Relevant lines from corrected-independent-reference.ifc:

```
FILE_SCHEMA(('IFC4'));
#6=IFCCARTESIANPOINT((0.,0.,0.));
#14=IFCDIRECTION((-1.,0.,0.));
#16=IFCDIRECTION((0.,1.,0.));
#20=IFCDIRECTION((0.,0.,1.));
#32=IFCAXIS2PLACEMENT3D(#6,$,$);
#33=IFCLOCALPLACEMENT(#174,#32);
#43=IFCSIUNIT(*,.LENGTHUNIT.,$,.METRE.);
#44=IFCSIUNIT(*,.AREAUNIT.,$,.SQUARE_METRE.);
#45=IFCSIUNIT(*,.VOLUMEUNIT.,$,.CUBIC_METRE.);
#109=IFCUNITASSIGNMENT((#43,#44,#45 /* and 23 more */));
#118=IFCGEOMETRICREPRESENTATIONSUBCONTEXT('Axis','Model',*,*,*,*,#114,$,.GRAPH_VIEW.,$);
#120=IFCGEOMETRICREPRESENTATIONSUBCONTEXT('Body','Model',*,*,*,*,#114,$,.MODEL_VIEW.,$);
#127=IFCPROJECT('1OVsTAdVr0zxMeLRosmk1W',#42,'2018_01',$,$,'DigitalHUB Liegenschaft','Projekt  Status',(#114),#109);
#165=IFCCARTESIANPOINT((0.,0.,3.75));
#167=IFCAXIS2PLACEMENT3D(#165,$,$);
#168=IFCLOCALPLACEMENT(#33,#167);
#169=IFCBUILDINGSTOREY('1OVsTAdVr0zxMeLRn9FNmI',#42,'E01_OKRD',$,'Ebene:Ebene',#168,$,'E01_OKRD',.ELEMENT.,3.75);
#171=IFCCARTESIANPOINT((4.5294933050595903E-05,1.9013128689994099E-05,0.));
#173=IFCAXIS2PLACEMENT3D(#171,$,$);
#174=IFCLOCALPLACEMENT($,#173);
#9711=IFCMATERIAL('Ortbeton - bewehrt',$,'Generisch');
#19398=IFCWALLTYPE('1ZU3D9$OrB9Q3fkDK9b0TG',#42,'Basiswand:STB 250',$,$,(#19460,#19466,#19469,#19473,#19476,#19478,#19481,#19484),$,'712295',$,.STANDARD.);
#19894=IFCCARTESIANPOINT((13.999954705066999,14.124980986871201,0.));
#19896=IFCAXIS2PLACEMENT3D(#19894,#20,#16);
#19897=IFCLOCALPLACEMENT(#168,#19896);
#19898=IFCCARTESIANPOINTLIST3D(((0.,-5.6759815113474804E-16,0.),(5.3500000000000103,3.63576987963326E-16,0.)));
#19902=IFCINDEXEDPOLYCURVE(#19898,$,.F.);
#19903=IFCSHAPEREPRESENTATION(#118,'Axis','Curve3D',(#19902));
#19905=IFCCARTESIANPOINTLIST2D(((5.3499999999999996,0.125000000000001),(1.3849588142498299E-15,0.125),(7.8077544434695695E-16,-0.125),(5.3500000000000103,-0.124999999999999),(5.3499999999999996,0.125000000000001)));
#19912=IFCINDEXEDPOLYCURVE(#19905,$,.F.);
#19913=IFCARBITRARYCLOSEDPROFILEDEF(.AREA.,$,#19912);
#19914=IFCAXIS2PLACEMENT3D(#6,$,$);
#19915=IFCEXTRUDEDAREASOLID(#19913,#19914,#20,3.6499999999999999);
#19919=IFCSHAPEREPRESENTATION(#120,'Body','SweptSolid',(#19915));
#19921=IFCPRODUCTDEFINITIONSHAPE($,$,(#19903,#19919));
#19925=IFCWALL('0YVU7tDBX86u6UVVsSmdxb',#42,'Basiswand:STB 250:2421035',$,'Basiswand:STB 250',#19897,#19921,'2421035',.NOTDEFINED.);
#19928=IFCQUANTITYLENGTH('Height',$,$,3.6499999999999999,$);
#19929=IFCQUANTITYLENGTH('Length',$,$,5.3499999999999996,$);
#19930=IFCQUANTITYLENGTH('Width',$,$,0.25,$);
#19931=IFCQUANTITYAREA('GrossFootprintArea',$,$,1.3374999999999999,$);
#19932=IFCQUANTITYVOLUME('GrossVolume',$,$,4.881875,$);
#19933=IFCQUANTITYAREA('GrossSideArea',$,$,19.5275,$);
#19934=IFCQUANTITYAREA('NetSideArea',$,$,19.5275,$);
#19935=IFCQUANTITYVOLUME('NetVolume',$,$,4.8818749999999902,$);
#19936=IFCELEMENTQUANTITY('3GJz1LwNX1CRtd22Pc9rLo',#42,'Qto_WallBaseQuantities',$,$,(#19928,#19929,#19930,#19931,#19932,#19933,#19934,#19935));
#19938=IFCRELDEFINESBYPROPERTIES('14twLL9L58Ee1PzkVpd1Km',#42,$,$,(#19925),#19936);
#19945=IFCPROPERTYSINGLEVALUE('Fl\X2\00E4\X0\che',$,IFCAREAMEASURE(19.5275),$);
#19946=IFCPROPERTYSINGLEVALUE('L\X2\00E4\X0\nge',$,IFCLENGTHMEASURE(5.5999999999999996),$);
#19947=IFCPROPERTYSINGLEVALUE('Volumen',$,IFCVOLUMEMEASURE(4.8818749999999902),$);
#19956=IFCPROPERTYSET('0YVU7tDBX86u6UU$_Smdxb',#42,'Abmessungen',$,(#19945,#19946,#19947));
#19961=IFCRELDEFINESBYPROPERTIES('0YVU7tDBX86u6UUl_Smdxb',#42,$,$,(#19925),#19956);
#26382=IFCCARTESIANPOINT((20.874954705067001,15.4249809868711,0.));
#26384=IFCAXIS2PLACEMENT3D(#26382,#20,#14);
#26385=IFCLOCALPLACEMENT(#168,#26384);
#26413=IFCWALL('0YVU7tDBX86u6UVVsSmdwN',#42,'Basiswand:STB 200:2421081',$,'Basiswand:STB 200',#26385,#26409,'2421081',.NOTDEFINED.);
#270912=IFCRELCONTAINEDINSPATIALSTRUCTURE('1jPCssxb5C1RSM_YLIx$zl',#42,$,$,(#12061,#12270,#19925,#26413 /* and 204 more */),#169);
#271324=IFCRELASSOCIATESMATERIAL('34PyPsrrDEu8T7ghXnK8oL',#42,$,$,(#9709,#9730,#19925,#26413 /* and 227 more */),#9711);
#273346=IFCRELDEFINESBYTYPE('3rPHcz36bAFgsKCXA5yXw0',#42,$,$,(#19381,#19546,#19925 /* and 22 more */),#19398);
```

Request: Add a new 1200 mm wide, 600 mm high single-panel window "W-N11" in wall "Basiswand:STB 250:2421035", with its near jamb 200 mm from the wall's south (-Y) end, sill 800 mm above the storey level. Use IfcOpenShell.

```python
import numpy as np
import ifcopenshell
import ifcopenshell.api.feature
import ifcopenshell.api.geometry
import ifcopenshell.api.pset
import ifcopenshell.api.root
import ifcopenshell.api.spatial
import ifcopenshell.geom
import ifcopenshell.util.element
import ifcopenshell.util.placement
import ifcopenshell.util.representation
import ifcopenshell.util.shape
import ifcopenshell.util.unit

model = ifcopenshell.open("corrected-independent-reference.ifc")
unit_scale = ifcopenshell.util.unit.calculate_unit_scale(model)
area_scale = ifcopenshell.util.unit.calculate_unit_scale(model, "AREAUNIT")
volume_scale = ifcopenshell.util.unit.calculate_unit_scale(model, "VOLUMEUNIT")
settings = ifcopenshell.geom.settings()


def volume(element):
    """Net volume in cubic metres, openings subtracted."""
    shape = ifcopenshell.geom.create_shape(settings, element)
    return ifcopenshell.util.shape.get_volume(shape.geometry)


wall = model.by_id(19925)
storey = ifcopenshell.util.element.get_container(wall, ifc_class="IfcBuildingStorey")
context = ifcopenshell.util.representation.get_context(model, "Model", "Body", "MODEL_VIEW")
before = volume(wall)

width, height, from_end, sill = 1.2, 0.6, 0.2, 0.8  # metres

# The wall runs along its own X axis, and the end named is its -X end.
wall_shape = ifcopenshell.geom.create_shape(settings, wall)
x, y, z = ifcopenshell.util.shape.get_vertices(wall_shape.geometry).T
start = x.min() + from_end
face, thickness = float(y.min()), float(y.max() - y.min())
wall_matrix = ifcopenshell.util.placement.get_local_placement(wall.ObjectPlacement)
level = ifcopenshell.util.placement.get_local_placement(storey.ObjectPlacement)[2, 3]


def in_wall(x, y):
    """Placement at x, y metres in the wall's axes, at sill height."""
    matrix = wall_matrix.copy()
    matrix[:, 3] = wall_matrix @ np.array([x / unit_scale, y / unit_scale, 0.0, 1.0])
    matrix[2, 3] = level + sill / unit_scale
    return matrix


# Opening: a box that overshoots both wall faces by 50 mm.
opening = ifcopenshell.api.root.create_entity(model, ifc_class="IfcOpeningElement", predefined_type="OPENING")
box = ifcopenshell.api.geometry.add_wall_representation(
    model, context=context, length=width, height=height, thickness=thickness + 0.1
)
ifcopenshell.api.geometry.assign_representation(model, product=opening, representation=box)
ifcopenshell.api.geometry.edit_object_placement(model, product=opening, matrix=in_wall(start, face - 0.05), is_si=False)
ifcopenshell.api.feature.add_feature(model, feature=opening, element=wall)

window = ifcopenshell.api.root.create_entity(model, ifc_class="IfcWindow", name="W-N11", predefined_type="WINDOW")
window.OverallWidth, window.OverallHeight = width / unit_scale, height / unit_scale
window.PartitioningType = "SINGLE_PANEL"
body = ifcopenshell.api.geometry.add_window_representation(
    model,
    context=context,
    overall_width=window.OverallWidth,
    overall_height=window.OverallHeight,
    partition_type="SINGLE_PANEL",
)
ifcopenshell.api.geometry.assign_representation(model, product=window, representation=body)
ifcopenshell.api.spatial.assign_container(model, products=[window], relating_structure=storey)
ifcopenshell.api.feature.add_filling(model, opening=opening, element=window)

# Centre the window in the wall's thickness.
ifcopenshell.api.geometry.edit_object_placement(model, product=window, matrix=in_wall(start, face), is_si=False)
window_shape = ifcopenshell.geom.create_shape(settings, window)
depth = ifcopenshell.util.shape.get_vertices(window_shape.geometry)[:, 1]
offset = face + thickness / 2 - (depth.min() + depth.max()) / 2
ifcopenshell.api.geometry.edit_object_placement(model, product=window, matrix=in_wall(start, offset), is_si=False)

after = volume(wall)

# Update the wall's stored quantities.
qto = model.by_id(ifcopenshell.util.element.get_pset(wall, "Qto_WallBaseQuantities", should_inherit=False)["id"])
ifcopenshell.api.pset.edit_qto(model, qto=qto, properties={
    "NetSideArea": after / thickness / area_scale,
    "NetVolume": after / volume_scale,
})
pset = model.by_id(ifcopenshell.util.element.get_pset(wall, "Abmessungen", should_inherit=False)["id"])
ifcopenshell.api.pset.edit_pset(model, pset=pset, properties={
    "Fläche": model.create_entity("IfcAreaMeasure", after / thickness / area_scale),
    "Volumen": model.create_entity("IfcVolumeMeasure", after / volume_scale),
})

print(f"wall volume {before:.3f} -> {after:.3f} m3")

model.write("corrected-independent-reference-out.ifc")
```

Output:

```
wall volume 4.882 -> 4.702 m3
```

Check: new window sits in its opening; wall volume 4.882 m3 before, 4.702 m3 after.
